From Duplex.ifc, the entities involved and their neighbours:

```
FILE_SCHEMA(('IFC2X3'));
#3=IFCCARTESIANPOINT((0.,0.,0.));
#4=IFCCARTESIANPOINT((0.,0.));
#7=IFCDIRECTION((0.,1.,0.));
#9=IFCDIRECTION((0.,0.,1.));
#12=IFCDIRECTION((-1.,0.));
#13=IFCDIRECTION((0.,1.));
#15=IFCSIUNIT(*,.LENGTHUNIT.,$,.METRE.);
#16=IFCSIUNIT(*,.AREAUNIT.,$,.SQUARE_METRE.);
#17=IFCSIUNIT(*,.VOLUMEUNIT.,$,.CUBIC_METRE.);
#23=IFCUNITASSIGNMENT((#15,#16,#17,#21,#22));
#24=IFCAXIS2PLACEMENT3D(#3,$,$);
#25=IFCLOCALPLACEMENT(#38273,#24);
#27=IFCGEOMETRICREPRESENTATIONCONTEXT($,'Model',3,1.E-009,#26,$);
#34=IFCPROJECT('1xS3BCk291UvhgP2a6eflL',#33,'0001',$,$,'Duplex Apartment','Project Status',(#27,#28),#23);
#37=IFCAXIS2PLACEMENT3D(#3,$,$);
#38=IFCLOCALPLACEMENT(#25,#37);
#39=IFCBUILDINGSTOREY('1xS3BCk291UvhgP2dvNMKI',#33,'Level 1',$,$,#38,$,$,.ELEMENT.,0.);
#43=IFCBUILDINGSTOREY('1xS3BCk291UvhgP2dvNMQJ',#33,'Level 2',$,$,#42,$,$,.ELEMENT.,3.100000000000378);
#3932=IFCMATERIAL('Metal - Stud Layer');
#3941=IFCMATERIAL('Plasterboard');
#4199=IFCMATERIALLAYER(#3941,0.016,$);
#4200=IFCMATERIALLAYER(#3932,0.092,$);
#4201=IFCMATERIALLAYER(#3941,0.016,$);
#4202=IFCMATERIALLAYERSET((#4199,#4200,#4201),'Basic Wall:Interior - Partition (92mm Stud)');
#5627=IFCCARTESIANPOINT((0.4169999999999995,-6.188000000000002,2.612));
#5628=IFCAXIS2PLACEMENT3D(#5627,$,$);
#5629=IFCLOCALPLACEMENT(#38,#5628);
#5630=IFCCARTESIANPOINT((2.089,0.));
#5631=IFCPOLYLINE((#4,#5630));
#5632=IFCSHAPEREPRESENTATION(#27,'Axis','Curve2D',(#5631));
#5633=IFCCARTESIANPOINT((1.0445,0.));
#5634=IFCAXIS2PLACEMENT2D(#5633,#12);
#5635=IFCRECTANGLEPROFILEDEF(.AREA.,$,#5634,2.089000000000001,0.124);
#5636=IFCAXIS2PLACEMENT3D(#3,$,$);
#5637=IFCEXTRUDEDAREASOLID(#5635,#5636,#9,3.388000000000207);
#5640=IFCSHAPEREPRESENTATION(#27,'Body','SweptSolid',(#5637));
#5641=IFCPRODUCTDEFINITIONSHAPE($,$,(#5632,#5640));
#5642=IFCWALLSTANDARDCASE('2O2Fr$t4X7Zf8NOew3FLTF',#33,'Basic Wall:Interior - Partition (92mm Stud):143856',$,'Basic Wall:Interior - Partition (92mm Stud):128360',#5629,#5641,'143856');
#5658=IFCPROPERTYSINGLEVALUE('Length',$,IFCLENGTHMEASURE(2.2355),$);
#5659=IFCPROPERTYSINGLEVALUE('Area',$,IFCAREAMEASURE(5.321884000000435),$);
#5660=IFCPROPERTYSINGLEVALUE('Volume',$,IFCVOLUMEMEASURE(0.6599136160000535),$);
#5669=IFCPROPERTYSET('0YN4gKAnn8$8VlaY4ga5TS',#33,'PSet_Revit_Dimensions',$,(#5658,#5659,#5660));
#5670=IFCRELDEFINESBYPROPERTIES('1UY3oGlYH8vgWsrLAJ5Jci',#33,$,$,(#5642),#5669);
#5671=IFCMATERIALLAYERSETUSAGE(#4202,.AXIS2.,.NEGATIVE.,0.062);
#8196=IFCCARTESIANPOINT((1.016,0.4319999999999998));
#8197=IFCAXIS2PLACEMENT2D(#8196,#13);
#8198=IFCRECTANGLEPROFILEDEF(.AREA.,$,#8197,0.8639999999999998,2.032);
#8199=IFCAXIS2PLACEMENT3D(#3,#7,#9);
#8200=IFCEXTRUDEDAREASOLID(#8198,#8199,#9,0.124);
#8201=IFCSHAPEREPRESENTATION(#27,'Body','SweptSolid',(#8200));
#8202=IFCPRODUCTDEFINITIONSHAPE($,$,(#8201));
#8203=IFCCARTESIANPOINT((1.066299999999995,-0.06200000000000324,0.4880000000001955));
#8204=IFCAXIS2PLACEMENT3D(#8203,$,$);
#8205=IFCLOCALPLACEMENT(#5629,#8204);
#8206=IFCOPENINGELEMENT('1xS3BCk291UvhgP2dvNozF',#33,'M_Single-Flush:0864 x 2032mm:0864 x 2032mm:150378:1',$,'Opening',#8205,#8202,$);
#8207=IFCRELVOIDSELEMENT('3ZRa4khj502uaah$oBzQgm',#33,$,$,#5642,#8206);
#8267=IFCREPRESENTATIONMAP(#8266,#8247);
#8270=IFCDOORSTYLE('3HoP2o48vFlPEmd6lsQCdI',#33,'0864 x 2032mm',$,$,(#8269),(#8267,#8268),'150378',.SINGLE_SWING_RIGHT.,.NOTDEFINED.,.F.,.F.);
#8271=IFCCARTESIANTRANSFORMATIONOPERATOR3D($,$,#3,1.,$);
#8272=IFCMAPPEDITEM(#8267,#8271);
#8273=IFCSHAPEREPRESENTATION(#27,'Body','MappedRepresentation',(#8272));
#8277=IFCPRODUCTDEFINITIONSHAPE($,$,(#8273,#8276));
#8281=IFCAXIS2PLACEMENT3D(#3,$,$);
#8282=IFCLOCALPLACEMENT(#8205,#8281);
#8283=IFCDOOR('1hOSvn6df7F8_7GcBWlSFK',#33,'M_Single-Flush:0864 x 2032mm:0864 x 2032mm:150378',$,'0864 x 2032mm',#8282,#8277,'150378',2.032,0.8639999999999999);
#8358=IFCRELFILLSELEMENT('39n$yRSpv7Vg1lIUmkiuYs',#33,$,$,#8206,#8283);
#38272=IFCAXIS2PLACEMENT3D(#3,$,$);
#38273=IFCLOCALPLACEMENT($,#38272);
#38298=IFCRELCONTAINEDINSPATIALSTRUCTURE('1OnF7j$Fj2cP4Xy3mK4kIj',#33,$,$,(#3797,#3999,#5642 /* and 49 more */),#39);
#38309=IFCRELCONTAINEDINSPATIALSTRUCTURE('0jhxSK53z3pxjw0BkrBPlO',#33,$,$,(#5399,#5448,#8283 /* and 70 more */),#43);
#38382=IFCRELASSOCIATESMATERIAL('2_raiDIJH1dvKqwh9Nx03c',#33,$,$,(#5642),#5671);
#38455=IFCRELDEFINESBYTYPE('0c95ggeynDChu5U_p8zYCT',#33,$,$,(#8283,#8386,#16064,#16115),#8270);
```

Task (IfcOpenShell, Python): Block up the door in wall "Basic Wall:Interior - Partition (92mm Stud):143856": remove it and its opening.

```python
import ifcopenshell
import ifcopenshell.api.feature
import ifcopenshell.api.pset
import ifcopenshell.api.root
import ifcopenshell.geom
import ifcopenshell.util.element
import ifcopenshell.util.shape
import ifcopenshell.util.unit

model = ifcopenshell.open("Duplex.ifc")
area_scale = ifcopenshell.util.unit.calculate_unit_scale(model, "AREAUNIT")
volume_scale = ifcopenshell.util.unit.calculate_unit_scale(model, "VOLUMEUNIT")
settings = ifcopenshell.geom.settings()


def volume(element):
    """Net volume in cubic metres, openings subtracted."""
    shape = ifcopenshell.geom.create_shape(settings, element)
    return ifcopenshell.util.shape.get_volume(shape.geometry)


door = model.by_guid("1hOSvn6df7F8_7GcBWlSFK")
opening = door.FillsVoids[0].RelatingOpeningElement
wall = opening.VoidsElements[0].RelatingBuildingElement
before = volume(wall)

ifcopenshell.api.root.remove_product(model, product=door)
ifcopenshell.api.feature.remove_feature(model, feature=opening)

after = volume(wall)
thickness = 0.124  # wall thickness in metres

# Update the wall's stored quantities.
pset = model.by_id(ifcopenshell.util.element.get_pset(wall, "PSet_Revit_Dimensions", should_inherit=False)["id"])
ifcopenshell.api.pset.edit_pset(model, pset=pset, properties={
    "Area": model.create_entity("IfcAreaMeasure", after / thickness / area_scale),
    "Volume": model.create_entity("IfcVolumeMeasure", after / volume_scale),
})

print(f"wall volume {before:.3f} -> {after:.3f} m3")

model.write("Duplex_v2.ifc")
```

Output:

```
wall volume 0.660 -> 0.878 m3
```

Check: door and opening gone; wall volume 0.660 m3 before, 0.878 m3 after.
